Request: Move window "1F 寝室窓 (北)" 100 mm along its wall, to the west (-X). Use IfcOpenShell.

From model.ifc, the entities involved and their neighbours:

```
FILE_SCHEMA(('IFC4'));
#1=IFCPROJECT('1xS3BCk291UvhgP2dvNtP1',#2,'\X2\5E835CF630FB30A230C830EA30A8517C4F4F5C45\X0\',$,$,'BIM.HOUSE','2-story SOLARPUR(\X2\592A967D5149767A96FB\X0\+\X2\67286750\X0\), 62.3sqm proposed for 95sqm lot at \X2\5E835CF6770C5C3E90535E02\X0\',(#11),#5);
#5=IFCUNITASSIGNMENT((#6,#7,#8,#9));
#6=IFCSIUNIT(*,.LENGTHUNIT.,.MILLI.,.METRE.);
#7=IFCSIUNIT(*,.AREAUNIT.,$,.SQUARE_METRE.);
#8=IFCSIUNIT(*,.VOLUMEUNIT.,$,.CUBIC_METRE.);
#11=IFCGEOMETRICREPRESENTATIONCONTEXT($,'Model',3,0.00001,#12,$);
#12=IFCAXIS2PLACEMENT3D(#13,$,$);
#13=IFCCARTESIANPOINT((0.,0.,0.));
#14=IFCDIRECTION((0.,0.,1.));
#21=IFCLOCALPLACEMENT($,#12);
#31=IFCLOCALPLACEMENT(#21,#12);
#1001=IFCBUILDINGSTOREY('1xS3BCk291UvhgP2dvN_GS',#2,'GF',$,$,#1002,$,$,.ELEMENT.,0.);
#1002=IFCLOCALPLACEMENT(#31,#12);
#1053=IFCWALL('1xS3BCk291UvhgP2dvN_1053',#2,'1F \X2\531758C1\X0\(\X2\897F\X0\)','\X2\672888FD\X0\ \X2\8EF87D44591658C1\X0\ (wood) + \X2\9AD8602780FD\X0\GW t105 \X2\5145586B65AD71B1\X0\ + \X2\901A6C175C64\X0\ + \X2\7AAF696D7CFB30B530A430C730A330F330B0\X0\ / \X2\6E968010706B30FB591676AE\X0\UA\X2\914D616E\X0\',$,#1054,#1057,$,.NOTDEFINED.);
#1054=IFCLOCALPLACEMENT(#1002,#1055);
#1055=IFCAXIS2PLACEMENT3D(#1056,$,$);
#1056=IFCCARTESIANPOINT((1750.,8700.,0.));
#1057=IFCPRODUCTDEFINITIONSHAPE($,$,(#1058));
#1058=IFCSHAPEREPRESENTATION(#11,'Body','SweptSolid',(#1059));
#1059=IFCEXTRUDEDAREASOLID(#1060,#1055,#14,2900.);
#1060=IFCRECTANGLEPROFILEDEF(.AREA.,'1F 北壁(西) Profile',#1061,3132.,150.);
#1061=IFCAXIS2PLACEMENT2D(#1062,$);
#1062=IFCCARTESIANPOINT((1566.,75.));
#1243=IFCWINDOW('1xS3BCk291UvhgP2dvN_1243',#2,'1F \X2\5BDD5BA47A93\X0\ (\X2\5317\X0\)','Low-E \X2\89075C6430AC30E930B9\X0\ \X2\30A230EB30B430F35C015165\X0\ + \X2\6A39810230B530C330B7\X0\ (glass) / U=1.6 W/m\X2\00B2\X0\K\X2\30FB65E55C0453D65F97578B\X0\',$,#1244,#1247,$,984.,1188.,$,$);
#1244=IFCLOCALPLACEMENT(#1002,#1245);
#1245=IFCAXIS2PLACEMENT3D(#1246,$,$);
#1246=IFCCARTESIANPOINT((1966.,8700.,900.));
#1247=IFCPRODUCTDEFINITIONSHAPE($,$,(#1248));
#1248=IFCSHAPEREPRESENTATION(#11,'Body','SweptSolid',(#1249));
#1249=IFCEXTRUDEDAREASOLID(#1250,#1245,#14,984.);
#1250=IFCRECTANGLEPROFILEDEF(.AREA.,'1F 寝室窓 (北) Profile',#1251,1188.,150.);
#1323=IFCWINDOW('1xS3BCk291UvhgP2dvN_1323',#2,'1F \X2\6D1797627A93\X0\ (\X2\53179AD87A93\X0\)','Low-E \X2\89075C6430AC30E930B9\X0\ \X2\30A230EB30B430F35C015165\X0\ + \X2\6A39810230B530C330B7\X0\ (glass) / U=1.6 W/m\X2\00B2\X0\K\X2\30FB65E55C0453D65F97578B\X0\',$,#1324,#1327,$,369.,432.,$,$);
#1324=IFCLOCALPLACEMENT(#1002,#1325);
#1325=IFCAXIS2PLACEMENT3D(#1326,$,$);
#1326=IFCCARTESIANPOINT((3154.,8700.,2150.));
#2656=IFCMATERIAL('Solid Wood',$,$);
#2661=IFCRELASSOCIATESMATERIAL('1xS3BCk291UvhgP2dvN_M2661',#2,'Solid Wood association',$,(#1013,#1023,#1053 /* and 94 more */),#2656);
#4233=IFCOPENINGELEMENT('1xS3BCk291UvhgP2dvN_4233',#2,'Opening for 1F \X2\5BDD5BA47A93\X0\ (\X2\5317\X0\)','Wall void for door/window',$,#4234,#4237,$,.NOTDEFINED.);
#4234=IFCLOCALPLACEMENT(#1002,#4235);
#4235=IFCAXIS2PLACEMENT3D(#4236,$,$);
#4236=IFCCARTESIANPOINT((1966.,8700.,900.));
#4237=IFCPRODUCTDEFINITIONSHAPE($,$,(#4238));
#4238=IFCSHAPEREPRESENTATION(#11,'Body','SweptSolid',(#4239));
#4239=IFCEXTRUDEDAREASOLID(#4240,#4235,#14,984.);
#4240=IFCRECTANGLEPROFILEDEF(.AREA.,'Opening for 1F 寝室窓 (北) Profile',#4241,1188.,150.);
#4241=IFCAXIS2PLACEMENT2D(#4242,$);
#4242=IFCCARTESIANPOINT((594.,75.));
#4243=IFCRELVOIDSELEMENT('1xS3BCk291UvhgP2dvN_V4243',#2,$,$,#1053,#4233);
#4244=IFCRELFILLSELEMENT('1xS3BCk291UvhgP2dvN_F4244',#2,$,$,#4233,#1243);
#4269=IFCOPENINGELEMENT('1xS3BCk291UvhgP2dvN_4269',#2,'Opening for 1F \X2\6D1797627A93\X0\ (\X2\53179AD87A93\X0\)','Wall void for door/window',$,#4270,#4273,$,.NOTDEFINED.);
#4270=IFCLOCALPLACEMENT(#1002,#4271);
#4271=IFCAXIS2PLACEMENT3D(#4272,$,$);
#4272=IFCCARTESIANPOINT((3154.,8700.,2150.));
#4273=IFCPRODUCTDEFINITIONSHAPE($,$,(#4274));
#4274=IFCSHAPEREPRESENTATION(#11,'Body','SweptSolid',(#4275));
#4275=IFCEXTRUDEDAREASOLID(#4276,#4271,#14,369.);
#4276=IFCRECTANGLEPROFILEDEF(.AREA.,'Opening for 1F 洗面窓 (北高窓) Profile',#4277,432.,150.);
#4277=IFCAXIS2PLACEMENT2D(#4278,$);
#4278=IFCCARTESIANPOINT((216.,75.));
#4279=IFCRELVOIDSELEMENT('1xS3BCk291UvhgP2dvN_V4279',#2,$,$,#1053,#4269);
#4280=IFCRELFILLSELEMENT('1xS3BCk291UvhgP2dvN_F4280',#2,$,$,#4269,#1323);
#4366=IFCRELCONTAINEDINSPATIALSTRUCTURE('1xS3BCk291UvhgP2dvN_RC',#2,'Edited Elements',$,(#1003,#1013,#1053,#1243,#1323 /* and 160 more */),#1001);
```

```python
import ifcopenshell
import ifcopenshell.api.geometry
import ifcopenshell.util.placement

model = ifcopenshell.open("model.ifc")

window = model.by_id(1243)
opening = window.FillsVoids[0].RelatingOpeningElement
wall = opening.VoidsElements[0].RelatingBuildingElement

wall_matrix = ifcopenshell.util.placement.get_local_placement(wall.ObjectPlacement)
shift = wall_matrix[:3, 0] * -100.0
before = ifcopenshell.util.placement.get_local_placement(window.ObjectPlacement)[:3, 3].copy()

# The window is not placed relative to its opening, so move both.
for product in (opening, window):
    matrix = ifcopenshell.util.placement.get_local_placement(product.ObjectPlacement)
    matrix[:3, 3] += shift
    ifcopenshell.api.geometry.edit_object_placement(model, product=product, matrix=matrix, is_si=False)

after = ifcopenshell.util.placement.get_local_placement(window.ObjectPlacement)[:3, 3]
print("window moved by", (after - before).round(3) + 0.0)

model.write("model_rev.ifc")
```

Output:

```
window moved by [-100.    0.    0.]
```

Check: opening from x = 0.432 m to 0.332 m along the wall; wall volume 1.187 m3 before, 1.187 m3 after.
